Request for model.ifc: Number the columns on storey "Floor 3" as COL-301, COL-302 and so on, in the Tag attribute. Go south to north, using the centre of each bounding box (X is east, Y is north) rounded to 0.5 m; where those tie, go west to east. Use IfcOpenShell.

First a look at what the model holds.

```python
import ifcopenshell
import ifcopenshell.util.element
import ifcopenshell.util.placement

model = ifcopenshell.open("model.ifc")
print(model.schema)
storey = next(s for s in model.by_type("IfcBuildingStorey") if s.Name == "Floor 3")
columns = [e for e in ifcopenshell.util.element.get_decomposition(storey) if e.is_a("IfcColumn")]
for e in sorted(columns, key=lambda e: e.id()):
    origin = ifcopenshell.util.placement.get_local_placement(e.ObjectPlacement)[:3, 3]
    print(e.id(), e.Tag, e.Name, origin.round(2) + 0.0, sep=" | ")
```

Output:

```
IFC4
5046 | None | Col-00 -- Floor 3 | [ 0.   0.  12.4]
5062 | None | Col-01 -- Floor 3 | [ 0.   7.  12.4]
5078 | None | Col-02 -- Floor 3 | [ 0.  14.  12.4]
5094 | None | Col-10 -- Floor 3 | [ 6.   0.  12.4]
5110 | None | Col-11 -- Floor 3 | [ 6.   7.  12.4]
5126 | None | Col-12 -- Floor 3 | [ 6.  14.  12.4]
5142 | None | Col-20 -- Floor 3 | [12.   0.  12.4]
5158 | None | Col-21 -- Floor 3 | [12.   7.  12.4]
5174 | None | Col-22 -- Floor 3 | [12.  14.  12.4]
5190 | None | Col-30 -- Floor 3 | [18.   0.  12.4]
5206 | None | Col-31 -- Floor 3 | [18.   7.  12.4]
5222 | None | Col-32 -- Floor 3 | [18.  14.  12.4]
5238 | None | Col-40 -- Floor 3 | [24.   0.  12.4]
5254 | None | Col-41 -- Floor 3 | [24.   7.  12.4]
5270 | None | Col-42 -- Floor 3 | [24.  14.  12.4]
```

```python
import ifcopenshell
import ifcopenshell.geom
import ifcopenshell.util.element
import ifcopenshell.util.shape

model = ifcopenshell.open("model.ifc")
settings = ifcopenshell.geom.settings()
settings.set("use-world-coords", True)


def centre(element):
    shape = ifcopenshell.geom.create_shape(settings, element)
    return ifcopenshell.util.shape.get_bbox_centroid(shape.geometry)


storey = next(s for s in model.by_type("IfcBuildingStorey") if s.Name == "Floor 3")
columns = [e for e in ifcopenshell.util.element.get_decomposition(storey) if e.is_a("IfcColumn")]

# Insertion points can sit at a corner or the storey origin, so sort by the geometry (in metres).
centres = {e: centre(e) for e in columns}
columns.sort(key=lambda e: (round(centres[e][1] / 0.5), centres[e][0]))

for i, e in enumerate(columns, start=1):
    number = f"COL-3{i:02d}"
    e.Tag = number
    print(e.id(), number)

model.write("model_rev.ifc")
```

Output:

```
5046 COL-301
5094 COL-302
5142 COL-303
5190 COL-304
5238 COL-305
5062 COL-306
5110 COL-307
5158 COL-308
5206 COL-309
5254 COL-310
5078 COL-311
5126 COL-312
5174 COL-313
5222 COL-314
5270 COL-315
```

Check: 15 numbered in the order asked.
